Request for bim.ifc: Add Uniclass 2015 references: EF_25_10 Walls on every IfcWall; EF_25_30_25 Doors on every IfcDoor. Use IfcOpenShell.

First a look at what the model holds.

```python
import ifcopenshell

model = ifcopenshell.open("bim.ifc")
print(model.schema)
print("classifications:", [c.Name for c in model.by_type("IfcClassification")])
for ifc_class in ("IfcDoor", "IfcRoof", "IfcStair", "IfcWall", "IfcWindow"):
    print(ifc_class, len(model.by_type(ifc_class)))
```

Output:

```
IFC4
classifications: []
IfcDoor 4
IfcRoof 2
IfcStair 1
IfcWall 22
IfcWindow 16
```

```python
import ifcopenshell
import ifcopenshell.api.classification

model = ifcopenshell.open("bim.ifc")

system = ifcopenshell.api.classification.add_classification(model, classification="Uniclass 2015")

codes = {
    "IfcWall": ("EF_25_10", "Walls"),
    "IfcDoor": ("EF_25_30_25", "Doors"),
}
for ifc_class, (code, name) in codes.items():
    products = model.by_type(ifc_class)
    ifcopenshell.api.classification.add_reference(
        model, products=products, classification=system, identification=code, name=name
    )
    print(code, len(products))

model.write("bim-out.ifc")
```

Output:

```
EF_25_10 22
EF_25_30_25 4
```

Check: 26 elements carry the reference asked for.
